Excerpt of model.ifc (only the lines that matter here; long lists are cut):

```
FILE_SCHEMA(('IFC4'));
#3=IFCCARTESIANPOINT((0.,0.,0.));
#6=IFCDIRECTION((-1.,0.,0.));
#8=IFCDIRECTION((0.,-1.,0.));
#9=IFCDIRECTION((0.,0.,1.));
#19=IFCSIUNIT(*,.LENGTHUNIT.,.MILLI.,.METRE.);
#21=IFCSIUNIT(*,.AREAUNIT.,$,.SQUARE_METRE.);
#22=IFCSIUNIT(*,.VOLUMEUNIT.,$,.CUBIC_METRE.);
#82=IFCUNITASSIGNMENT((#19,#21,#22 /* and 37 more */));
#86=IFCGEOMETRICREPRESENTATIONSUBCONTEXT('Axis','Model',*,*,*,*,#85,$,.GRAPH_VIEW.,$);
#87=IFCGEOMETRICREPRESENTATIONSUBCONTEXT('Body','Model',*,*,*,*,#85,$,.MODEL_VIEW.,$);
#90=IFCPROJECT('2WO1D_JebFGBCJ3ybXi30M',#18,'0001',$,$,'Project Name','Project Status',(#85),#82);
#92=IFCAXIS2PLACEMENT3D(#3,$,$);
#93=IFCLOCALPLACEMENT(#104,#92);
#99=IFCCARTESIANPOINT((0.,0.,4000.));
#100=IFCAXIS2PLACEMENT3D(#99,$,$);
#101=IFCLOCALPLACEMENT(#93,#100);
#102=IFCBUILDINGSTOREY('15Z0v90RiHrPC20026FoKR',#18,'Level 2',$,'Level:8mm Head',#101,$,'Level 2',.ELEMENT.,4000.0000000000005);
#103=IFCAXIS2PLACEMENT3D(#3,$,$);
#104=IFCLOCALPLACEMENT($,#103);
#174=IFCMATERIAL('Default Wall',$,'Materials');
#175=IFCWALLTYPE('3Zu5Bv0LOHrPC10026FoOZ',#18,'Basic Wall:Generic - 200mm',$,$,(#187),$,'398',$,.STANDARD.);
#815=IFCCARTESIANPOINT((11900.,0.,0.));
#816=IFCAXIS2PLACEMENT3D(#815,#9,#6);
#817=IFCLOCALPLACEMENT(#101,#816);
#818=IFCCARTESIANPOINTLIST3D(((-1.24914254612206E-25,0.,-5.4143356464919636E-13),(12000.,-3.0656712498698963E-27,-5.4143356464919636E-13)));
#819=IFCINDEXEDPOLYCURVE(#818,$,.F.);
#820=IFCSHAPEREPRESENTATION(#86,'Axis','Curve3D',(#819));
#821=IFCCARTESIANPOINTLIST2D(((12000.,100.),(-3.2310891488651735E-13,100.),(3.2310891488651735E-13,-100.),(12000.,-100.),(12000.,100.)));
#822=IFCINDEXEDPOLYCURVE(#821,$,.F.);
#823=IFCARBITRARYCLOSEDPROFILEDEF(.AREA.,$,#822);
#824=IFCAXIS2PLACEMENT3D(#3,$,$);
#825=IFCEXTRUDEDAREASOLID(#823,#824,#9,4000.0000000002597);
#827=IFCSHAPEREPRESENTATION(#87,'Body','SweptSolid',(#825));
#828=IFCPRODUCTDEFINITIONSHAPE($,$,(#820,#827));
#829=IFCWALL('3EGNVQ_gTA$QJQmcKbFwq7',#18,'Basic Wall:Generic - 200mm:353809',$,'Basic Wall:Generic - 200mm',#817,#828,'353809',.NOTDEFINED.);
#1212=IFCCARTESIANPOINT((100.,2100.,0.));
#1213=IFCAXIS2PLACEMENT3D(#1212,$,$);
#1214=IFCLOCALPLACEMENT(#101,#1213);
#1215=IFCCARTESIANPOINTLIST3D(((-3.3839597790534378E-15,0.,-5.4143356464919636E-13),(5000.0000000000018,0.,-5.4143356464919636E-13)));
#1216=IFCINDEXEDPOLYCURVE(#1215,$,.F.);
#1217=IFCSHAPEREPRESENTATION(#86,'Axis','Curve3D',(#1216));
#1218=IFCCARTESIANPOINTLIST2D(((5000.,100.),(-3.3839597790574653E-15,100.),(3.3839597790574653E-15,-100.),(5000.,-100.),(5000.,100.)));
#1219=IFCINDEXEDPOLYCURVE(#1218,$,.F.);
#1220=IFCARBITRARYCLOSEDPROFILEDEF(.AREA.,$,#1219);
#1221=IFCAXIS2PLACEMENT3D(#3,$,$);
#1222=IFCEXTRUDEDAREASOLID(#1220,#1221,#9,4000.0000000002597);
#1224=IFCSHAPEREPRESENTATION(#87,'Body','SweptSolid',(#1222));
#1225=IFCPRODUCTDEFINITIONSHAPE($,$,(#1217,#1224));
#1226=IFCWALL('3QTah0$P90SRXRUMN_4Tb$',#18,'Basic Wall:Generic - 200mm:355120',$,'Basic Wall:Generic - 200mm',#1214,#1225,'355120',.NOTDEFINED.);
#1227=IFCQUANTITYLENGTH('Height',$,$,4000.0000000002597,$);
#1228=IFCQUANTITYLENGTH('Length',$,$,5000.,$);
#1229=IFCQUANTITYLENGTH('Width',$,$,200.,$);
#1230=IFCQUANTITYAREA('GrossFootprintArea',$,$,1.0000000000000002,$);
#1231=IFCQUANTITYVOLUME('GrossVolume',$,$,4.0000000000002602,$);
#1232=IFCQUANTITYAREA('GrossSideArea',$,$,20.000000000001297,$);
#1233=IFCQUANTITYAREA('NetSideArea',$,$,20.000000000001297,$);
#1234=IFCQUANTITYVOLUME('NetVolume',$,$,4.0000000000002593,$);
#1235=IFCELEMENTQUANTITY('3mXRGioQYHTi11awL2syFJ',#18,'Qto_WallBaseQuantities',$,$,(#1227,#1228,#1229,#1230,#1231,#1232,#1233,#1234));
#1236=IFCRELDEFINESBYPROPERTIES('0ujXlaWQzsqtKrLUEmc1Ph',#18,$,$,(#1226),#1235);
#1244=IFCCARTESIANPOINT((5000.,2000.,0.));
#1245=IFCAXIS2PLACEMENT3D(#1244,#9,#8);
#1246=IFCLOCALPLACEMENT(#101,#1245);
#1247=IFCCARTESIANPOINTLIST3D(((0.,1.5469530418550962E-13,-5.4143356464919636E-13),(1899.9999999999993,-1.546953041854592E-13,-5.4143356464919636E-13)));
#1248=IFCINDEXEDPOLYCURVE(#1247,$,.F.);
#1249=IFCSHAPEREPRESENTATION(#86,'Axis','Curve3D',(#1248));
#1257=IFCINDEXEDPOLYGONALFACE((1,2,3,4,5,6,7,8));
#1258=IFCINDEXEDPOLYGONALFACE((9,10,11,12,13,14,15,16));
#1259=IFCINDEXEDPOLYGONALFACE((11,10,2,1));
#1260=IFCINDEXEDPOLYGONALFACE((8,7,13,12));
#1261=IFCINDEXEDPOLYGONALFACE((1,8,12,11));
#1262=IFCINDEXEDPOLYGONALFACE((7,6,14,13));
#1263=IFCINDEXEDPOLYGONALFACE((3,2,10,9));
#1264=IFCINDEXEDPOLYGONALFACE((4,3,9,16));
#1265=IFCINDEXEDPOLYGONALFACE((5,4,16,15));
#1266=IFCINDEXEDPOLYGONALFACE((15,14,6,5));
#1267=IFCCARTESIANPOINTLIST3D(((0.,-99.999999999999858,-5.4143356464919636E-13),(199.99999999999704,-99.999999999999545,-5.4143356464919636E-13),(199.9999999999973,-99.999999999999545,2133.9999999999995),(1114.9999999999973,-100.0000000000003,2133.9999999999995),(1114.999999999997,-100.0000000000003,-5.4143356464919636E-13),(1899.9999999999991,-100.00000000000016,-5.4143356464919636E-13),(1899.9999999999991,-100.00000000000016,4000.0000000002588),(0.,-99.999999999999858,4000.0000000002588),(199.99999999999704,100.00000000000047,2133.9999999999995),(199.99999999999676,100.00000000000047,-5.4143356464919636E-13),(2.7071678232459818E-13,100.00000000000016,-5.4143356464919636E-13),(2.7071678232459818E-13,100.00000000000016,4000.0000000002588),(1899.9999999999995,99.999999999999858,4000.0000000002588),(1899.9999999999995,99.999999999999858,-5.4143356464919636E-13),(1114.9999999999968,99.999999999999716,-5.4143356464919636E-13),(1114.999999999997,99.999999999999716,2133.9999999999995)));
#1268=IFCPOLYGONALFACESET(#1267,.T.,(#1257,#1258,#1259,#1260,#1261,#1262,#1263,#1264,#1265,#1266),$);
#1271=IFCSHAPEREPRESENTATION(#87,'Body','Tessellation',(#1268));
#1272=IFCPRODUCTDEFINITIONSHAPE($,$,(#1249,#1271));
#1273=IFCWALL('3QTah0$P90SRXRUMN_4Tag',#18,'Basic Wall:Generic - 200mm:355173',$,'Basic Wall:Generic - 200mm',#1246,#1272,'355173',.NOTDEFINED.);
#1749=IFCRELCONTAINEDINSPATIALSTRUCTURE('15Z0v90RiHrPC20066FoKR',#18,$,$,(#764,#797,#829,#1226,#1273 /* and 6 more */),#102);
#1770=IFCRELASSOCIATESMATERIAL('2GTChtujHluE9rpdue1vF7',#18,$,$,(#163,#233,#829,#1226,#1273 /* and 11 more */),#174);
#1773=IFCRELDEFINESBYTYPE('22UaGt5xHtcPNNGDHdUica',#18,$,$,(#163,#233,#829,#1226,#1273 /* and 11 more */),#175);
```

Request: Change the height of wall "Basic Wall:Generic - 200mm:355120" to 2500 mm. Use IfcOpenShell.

```python
import ifcopenshell
import ifcopenshell.api.pset
import ifcopenshell.geom
import ifcopenshell.util.element
import ifcopenshell.util.representation
import ifcopenshell.util.shape
import ifcopenshell.util.unit

model = ifcopenshell.open("model.ifc")
unit_scale = ifcopenshell.util.unit.calculate_unit_scale(model)
area_scale = ifcopenshell.util.unit.calculate_unit_scale(model, "AREAUNIT")
volume_scale = ifcopenshell.util.unit.calculate_unit_scale(model, "VOLUMEUNIT")
settings = ifcopenshell.geom.settings()


def volume(element):
    """Net volume in cubic metres, openings subtracted."""
    shape = ifcopenshell.geom.create_shape(settings, element)
    return ifcopenshell.util.shape.get_volume(shape.geometry)


wall = model.by_guid("3QTah0$P90SRXRUMN_4Tb$")
before = volume(wall)

body = ifcopenshell.util.representation.get_representation(wall, "Model", "Body")
solid = body.Items[0]
old_height = solid.Depth
solid.Depth = 2500.0
after = volume(wall)
thickness = 0.2  # wall thickness in metres

# Update the stored height, areas and volumes.
qto = model.by_id(ifcopenshell.util.element.get_pset(wall, "Qto_WallBaseQuantities", should_inherit=False)["id"])
ifcopenshell.api.pset.edit_qto(model, qto=qto, properties={
    "Height": solid.Depth,
    "GrossVolume": ifcopenshell.util.element.get_pset(wall, "Qto_WallBaseQuantities", "GrossVolume") * solid.Depth / old_height,
    "GrossSideArea": ifcopenshell.util.element.get_pset(wall, "Qto_WallBaseQuantities", "GrossSideArea") * solid.Depth / old_height,
    "NetSideArea": after / thickness / area_scale,
    "NetVolume": after / volume_scale,
})

print(f"height {old_height:g} -> {solid.Depth:g}, volume {before:.3f} -> {after:.3f} m3")

model.write("model_v2.ifc")
```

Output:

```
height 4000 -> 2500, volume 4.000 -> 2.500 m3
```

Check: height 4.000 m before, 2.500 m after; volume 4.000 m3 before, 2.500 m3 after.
